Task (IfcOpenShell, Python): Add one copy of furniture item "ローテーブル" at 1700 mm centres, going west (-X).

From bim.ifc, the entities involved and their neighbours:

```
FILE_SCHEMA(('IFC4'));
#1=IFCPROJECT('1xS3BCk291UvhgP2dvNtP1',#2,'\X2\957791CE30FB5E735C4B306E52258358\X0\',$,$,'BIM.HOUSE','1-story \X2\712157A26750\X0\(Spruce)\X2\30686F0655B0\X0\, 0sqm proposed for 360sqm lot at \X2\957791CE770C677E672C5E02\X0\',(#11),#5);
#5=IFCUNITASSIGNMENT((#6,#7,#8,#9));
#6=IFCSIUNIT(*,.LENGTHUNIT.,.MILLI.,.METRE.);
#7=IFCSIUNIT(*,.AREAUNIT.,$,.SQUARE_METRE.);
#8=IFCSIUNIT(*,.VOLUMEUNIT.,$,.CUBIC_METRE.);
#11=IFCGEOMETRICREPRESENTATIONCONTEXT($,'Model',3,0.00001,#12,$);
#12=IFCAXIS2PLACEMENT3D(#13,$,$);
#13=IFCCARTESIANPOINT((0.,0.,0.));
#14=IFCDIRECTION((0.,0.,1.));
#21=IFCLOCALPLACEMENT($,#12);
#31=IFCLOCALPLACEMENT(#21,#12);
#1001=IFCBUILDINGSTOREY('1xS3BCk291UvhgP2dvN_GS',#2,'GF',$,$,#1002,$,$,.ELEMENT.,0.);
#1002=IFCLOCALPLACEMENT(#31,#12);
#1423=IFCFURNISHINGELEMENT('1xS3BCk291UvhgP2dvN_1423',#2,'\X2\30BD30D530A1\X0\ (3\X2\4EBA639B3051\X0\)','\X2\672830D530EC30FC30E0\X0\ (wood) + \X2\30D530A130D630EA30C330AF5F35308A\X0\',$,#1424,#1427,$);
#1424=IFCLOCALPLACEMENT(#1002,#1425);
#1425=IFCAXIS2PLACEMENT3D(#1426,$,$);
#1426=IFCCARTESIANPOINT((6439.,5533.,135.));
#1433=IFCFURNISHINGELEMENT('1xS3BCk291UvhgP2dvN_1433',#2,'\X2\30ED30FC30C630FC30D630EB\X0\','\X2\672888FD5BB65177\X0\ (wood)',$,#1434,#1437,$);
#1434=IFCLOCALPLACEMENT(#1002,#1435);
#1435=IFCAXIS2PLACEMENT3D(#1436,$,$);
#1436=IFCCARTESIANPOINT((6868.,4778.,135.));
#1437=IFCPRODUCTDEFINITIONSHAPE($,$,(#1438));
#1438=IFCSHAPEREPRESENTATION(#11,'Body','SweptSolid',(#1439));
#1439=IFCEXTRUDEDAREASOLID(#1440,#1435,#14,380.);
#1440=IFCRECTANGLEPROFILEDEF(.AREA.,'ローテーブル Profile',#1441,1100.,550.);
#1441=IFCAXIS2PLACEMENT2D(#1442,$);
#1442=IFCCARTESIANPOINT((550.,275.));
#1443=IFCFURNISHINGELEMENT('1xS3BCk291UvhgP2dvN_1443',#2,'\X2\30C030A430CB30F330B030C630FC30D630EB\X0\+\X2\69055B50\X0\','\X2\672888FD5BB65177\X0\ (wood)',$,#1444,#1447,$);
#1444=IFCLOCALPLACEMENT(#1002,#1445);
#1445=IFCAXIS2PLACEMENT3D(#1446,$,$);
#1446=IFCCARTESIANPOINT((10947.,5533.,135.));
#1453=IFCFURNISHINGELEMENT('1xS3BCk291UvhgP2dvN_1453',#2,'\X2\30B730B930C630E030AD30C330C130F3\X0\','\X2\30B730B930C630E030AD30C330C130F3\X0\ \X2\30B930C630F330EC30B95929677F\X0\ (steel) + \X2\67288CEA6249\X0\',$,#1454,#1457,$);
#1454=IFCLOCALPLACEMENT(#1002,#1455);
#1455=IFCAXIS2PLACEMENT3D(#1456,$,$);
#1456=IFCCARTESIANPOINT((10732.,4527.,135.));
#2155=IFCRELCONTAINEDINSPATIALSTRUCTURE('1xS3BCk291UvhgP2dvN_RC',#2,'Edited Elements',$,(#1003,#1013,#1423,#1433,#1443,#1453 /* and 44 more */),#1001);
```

```python
import numpy as np
import ifcopenshell
import ifcopenshell.api.geometry
import ifcopenshell.api.root
import ifcopenshell.util.element
import ifcopenshell.util.placement

model = ifcopenshell.open("bim.ifc")


def reuse_history(source, copy):
    """copy_class also copies each property set's owner history, people and application; keep the originals."""
    for rel in copy.IsDefinedBy:
        if rel.is_a("IfcRelDefinesByProperties") and (history := rel.RelatingPropertyDefinition.OwnerHistory):
            rel.RelatingPropertyDefinition.OwnerHistory = source.OwnerHistory
            ifcopenshell.util.element.remove_deep2(model, history)


source = model.by_id(1433)
base = ifcopenshell.util.placement.get_local_placement(source.ObjectPlacement)
step = np.array([-1.0, 0.0, 0.0]) * 1700.0

for i in range(1, 2):
    copy = ifcopenshell.api.root.copy_class(model, product=source)
    copy.Representation = ifcopenshell.util.element.copy_deep(
        model, source.Representation, exclude=["IfcGeometricRepresentationContext", "IfcRepresentationMap"]
    )
    reuse_history(source, copy)
    matrix = base.copy()
    matrix[:3, 3] += i * step
    print("added at", matrix[:3, 3].round(3) + 0.0)
    ifcopenshell.api.geometry.edit_object_placement(model, product=copy, matrix=matrix, is_si=False)

model.write("bim_edited.ifc")
```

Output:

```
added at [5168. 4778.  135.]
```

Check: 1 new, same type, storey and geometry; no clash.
